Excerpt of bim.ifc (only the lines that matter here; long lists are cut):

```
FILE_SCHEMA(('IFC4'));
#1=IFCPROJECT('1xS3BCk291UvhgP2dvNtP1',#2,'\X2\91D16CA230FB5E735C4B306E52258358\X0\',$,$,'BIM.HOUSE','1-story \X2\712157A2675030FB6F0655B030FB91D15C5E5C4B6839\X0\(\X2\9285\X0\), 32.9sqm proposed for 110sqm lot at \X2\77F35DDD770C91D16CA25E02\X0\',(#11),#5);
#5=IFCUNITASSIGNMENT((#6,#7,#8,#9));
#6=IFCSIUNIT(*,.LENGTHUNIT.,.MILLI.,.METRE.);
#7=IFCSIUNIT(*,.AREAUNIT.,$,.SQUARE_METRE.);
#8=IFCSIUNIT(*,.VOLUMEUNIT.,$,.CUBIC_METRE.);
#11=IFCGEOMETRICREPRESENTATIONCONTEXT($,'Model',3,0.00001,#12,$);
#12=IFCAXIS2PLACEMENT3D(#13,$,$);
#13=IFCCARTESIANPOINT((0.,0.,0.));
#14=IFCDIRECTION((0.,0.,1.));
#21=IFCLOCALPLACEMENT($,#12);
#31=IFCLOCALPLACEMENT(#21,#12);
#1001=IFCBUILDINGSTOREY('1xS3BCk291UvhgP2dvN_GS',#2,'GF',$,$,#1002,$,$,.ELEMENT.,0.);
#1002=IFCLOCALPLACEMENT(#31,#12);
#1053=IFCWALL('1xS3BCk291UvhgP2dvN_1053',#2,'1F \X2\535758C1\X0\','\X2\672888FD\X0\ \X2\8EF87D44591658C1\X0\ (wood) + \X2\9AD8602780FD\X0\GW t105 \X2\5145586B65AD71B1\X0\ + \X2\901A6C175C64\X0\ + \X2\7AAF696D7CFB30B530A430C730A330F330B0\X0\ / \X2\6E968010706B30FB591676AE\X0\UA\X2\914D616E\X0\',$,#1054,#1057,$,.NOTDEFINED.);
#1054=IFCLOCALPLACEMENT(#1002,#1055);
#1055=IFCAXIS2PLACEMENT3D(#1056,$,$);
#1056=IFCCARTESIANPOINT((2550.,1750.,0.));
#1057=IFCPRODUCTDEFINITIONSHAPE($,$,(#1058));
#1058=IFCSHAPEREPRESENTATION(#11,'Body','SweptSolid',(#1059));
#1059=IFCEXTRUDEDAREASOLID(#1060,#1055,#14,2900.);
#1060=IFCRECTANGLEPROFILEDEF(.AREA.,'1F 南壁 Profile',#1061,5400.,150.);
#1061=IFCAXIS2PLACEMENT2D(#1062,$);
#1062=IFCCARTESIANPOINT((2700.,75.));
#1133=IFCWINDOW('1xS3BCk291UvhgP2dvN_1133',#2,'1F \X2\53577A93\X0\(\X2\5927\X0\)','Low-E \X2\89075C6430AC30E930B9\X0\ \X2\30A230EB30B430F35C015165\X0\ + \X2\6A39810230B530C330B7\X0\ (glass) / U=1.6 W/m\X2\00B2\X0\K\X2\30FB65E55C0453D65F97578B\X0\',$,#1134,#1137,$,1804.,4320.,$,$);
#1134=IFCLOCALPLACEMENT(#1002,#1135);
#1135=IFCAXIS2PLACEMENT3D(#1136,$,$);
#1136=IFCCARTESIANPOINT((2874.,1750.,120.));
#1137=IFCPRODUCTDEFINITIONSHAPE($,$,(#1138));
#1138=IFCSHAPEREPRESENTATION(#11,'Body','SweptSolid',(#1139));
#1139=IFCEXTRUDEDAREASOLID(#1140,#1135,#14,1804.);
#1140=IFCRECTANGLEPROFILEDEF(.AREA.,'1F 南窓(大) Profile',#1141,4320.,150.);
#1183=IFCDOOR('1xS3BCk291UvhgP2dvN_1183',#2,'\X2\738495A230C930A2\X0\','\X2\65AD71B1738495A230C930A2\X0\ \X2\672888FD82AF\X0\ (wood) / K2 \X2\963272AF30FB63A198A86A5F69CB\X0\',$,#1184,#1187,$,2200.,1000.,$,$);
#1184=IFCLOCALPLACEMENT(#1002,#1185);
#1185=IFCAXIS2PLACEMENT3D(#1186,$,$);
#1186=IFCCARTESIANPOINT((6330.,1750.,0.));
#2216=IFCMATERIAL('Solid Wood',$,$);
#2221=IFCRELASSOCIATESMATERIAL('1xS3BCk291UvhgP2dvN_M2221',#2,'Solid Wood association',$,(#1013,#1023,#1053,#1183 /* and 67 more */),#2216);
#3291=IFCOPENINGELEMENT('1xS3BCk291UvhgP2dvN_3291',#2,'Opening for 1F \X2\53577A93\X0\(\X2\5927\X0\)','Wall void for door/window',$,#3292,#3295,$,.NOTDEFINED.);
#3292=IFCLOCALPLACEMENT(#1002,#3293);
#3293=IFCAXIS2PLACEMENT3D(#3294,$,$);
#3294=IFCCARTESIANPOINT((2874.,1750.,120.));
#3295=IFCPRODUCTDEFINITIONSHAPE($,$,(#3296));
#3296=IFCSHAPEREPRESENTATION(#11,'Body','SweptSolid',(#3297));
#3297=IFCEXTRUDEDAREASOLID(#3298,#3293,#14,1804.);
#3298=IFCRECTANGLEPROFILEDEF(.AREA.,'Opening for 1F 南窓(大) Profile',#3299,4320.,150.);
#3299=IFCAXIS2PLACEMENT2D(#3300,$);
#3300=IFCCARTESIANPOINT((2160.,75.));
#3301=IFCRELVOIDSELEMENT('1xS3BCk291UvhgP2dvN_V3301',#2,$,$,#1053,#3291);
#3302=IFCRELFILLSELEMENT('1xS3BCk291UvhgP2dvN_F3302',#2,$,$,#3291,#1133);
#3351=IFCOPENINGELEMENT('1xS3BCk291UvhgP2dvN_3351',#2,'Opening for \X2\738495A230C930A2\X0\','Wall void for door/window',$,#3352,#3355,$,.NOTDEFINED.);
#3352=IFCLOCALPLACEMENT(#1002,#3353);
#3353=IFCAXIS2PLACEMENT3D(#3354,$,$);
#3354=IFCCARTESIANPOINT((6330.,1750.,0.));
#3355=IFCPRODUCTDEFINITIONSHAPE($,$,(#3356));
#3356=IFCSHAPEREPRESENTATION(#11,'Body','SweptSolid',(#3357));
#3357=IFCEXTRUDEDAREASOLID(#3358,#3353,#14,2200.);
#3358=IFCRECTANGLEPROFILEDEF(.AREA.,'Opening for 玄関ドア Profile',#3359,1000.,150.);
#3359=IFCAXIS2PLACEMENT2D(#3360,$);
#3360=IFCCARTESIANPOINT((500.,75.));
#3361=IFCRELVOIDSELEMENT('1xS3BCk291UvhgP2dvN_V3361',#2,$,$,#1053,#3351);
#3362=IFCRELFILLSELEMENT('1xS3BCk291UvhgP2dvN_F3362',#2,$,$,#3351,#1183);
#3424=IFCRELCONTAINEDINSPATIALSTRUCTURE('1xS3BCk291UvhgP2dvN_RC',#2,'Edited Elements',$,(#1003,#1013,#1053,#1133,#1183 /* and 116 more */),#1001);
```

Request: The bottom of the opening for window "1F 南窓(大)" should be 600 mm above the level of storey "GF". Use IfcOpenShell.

```python
import numpy as np
import ifcopenshell
import ifcopenshell.api.geometry
import ifcopenshell.geom
import ifcopenshell.util.element
import ifcopenshell.util.placement
import ifcopenshell.util.shape
import ifcopenshell.util.unit

model = ifcopenshell.open("bim.ifc")
unit_scale = ifcopenshell.util.unit.calculate_unit_scale(model)

window = model.by_id(1133)
opening = window.FillsVoids[0].RelatingOpeningElement
storey = ifcopenshell.util.element.get_container(window, ifc_class="IfcBuildingStorey")
level = ifcopenshell.util.placement.get_local_placement(storey.ObjectPlacement)[2, 3]

# The opening's origin need not be at the sill, so measure its lowest point.
shape = ifcopenshell.geom.create_shape(ifcopenshell.geom.settings(), opening)
bottom = ifcopenshell.util.shape.get_shape_bottom_elevation(shape, shape.geometry) / unit_scale
dz = level + 0.6 / unit_scale - bottom

shift = np.array([0.0, 0.0, dz])
# The window is not placed relative to its opening, so move both.
for product in (opening, window):
    matrix = ifcopenshell.util.placement.get_local_placement(product.ObjectPlacement)
    matrix[:3, 3] += shift
    ifcopenshell.api.geometry.edit_object_placement(model, product=product, matrix=matrix, is_si=False)

print(f"moved by {dz * unit_scale:+.3f} m")

model.write("bim-out.ifc")
```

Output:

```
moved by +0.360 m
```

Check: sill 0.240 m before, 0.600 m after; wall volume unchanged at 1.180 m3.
